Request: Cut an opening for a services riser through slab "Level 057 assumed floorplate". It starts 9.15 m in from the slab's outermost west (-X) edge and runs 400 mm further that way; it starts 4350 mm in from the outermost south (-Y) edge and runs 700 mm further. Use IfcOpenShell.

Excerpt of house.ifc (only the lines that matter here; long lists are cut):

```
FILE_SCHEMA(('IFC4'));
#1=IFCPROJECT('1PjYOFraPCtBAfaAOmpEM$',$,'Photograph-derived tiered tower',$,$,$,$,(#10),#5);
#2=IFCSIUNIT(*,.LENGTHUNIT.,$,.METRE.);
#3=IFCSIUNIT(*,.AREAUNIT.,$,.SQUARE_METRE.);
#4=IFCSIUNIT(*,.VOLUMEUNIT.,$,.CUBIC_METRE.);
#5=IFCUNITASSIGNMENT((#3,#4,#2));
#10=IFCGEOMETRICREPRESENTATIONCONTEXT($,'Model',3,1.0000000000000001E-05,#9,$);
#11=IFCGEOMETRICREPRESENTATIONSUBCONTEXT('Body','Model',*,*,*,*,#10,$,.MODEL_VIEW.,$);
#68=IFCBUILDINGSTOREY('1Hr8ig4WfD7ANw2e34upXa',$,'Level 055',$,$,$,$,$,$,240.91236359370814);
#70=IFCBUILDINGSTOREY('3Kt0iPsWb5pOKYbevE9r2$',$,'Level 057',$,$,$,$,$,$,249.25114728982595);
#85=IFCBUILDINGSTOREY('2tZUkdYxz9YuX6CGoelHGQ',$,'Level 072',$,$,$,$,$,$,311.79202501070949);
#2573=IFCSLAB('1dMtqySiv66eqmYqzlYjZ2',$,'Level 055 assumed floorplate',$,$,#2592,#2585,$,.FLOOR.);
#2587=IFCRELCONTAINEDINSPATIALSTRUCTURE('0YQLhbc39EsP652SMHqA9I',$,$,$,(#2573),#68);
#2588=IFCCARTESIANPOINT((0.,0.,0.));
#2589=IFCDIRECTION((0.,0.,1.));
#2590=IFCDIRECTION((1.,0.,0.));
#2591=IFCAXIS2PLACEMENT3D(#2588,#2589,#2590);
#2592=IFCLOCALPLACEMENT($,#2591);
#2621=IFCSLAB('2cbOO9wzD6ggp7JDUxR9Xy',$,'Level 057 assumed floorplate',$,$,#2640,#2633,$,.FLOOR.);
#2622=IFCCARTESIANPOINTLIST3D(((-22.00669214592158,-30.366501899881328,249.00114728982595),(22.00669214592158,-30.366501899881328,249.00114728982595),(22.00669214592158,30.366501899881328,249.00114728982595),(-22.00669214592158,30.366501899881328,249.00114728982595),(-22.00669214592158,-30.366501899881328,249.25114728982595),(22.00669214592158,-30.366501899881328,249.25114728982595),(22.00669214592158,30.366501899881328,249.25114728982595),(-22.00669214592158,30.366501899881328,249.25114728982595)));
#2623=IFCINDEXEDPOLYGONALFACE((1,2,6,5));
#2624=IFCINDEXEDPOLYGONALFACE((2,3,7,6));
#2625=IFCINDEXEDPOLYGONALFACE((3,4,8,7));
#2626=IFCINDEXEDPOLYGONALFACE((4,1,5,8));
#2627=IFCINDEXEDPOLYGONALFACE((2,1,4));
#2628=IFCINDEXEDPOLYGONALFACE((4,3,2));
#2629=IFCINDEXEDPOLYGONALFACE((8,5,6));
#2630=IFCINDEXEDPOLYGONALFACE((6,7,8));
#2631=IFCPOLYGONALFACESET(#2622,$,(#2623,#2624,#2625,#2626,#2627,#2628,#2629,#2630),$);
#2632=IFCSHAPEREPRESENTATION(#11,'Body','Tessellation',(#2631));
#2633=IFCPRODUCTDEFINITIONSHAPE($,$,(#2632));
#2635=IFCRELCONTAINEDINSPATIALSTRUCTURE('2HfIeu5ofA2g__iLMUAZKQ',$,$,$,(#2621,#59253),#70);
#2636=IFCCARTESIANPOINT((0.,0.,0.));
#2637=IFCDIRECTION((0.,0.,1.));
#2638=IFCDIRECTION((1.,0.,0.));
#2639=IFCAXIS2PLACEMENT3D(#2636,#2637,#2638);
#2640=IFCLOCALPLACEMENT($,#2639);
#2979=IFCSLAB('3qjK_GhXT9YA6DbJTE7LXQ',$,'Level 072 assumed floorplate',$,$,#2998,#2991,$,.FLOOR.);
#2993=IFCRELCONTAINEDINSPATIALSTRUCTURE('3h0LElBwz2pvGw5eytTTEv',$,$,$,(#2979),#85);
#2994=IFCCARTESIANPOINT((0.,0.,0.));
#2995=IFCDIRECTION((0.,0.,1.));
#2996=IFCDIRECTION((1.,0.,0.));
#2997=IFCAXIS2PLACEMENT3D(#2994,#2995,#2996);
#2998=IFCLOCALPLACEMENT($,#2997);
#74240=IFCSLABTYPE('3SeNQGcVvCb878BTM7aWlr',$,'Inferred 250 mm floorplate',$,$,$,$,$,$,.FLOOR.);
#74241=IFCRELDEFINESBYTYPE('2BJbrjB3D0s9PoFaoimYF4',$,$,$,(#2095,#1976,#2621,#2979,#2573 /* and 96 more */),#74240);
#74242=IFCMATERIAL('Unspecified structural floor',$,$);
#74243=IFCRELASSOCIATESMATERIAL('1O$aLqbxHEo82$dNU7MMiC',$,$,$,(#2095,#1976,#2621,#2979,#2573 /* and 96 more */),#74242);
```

```python
import numpy as np
import ifcopenshell
import ifcopenshell.api.feature
import ifcopenshell.api.geometry
import ifcopenshell.api.root
import ifcopenshell.geom
import ifcopenshell.util.placement
import ifcopenshell.util.representation
import ifcopenshell.util.shape
import ifcopenshell.util.unit

model = ifcopenshell.open("house.ifc")
unit_scale = ifcopenshell.util.unit.calculate_unit_scale(model)
settings = ifcopenshell.geom.settings()


def volume(element):
    """Net volume in cubic metres, openings subtracted."""
    shape = ifcopenshell.geom.create_shape(settings, element)
    return ifcopenshell.util.shape.get_volume(shape.geometry)


slab = model.by_id(2621)
before = volume(slab)

# Extent in the slab's own axes, in metres. The edges named are its -X and -Y sides.
slab_shape = ifcopenshell.geom.create_shape(settings, slab)
vertices = ifcopenshell.util.shape.get_vertices(slab_shape.geometry)
x_min, y_min, bottom = vertices.min(axis=0)
top = vertices[:, 2].max()

opening = ifcopenshell.api.root.create_entity(model, ifc_class="IfcOpeningElement", name="Services riser opening", predefined_type="OPENING")
context = ifcopenshell.util.representation.get_context(model, "Model", "Body", "MODEL_VIEW")
width, depth = 0.4, 0.7
outline = [(0.0, 0.0), (width, 0.0), (width, depth), (0.0, depth), (0.0, 0.0)]
# Overshoot both faces by 50 mm so the cut is clean.
shape = ifcopenshell.api.geometry.add_slab_representation(
    model, context=context, depth=top - bottom + 0.1, polyline=outline
)
ifcopenshell.api.geometry.assign_representation(model, product=opening, representation=shape)

matrix = ifcopenshell.util.placement.get_local_placement(slab.ObjectPlacement)
matrix[:, 3] = matrix @ np.append(np.array([x_min + 9.15, y_min + 4.35, bottom - 0.05]) / unit_scale, 1.0)
ifcopenshell.api.geometry.edit_object_placement(model, product=opening, matrix=matrix, is_si=False)
ifcopenshell.api.feature.add_feature(model, feature=opening, element=slab)

after = volume(slab)

print(f"slab volume {before:.3f} -> {after:.3f} m3")

model.write("house_rev.ifc")
```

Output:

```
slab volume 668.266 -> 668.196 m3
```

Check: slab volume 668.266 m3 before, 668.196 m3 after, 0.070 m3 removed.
